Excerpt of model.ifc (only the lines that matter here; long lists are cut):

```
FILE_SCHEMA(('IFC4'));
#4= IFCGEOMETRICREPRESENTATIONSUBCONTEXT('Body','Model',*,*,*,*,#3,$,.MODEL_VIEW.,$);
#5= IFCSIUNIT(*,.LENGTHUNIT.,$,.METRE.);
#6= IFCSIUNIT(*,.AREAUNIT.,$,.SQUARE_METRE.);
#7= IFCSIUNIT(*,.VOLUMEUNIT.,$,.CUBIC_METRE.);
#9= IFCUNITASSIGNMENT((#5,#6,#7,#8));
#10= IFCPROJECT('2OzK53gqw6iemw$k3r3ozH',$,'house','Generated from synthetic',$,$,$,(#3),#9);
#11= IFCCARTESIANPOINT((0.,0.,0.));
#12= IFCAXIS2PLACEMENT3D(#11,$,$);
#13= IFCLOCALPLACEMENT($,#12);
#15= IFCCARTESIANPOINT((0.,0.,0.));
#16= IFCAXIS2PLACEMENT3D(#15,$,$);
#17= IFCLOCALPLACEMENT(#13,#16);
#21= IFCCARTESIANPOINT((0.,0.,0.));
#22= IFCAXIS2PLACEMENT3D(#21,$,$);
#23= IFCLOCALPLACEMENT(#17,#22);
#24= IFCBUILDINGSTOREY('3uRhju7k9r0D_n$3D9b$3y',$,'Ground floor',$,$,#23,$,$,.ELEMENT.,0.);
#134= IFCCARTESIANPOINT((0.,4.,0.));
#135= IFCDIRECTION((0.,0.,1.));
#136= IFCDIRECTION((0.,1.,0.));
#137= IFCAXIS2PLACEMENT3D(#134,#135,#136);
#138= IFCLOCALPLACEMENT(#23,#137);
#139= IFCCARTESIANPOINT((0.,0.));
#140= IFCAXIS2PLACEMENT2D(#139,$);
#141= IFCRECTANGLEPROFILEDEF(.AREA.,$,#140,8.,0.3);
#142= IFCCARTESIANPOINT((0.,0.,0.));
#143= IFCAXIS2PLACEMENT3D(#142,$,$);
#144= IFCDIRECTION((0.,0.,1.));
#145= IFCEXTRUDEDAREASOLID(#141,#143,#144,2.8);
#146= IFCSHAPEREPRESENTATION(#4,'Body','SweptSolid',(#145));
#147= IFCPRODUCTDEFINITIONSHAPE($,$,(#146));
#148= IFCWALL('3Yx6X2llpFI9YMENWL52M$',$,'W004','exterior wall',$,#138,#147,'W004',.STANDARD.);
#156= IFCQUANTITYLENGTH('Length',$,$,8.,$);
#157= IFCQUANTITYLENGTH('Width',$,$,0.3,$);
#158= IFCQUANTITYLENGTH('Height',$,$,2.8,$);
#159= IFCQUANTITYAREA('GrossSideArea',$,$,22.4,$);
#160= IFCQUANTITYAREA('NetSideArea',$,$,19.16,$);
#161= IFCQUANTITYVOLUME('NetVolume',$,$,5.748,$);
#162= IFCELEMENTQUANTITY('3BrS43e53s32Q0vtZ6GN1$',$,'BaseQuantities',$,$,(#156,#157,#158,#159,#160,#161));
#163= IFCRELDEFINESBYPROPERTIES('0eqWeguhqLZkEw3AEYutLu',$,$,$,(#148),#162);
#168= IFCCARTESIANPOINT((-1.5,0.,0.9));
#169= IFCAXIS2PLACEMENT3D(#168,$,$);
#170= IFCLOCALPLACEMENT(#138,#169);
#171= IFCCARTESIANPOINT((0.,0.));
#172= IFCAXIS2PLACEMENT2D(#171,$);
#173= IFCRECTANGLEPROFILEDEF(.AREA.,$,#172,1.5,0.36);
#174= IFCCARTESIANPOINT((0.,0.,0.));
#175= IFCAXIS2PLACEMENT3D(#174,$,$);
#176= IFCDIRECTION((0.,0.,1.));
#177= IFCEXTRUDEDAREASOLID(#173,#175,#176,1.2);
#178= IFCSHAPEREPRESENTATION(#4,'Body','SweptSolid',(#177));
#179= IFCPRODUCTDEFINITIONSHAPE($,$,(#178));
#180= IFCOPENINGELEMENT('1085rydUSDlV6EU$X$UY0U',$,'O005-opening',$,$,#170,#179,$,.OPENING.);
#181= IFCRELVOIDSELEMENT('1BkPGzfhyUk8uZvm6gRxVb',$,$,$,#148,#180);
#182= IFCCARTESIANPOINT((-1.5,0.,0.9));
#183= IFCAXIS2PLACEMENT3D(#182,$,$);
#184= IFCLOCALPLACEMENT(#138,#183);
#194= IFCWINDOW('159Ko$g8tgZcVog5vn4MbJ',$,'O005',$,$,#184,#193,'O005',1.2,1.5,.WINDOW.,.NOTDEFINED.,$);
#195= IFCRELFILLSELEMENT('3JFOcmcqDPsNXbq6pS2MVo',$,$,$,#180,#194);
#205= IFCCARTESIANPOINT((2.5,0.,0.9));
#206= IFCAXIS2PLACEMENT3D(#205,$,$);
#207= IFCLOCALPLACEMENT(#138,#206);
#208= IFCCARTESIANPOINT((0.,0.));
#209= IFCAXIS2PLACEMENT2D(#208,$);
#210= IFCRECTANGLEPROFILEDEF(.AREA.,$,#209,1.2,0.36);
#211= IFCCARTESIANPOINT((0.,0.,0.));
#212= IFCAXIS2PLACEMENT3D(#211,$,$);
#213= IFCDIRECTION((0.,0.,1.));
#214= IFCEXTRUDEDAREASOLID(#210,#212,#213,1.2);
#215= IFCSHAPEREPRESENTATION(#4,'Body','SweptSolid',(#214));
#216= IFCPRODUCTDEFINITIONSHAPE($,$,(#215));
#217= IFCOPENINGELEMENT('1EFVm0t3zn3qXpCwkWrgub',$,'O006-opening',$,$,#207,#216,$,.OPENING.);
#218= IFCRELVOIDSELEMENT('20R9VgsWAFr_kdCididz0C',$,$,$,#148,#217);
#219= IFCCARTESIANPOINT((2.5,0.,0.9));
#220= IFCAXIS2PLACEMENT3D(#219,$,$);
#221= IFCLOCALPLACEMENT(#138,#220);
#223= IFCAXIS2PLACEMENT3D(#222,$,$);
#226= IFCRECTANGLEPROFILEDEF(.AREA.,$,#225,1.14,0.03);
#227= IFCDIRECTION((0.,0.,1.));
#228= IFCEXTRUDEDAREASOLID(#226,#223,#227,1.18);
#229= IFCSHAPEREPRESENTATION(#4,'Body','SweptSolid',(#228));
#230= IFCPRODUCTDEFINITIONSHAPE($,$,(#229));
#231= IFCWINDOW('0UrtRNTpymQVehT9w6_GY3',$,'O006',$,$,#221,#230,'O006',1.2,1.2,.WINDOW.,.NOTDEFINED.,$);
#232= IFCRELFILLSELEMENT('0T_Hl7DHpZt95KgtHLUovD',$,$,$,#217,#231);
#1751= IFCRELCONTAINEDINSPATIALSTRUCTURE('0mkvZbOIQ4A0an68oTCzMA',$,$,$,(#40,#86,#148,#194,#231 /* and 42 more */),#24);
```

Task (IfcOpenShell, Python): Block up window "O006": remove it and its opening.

```python
import ifcopenshell
import ifcopenshell.api.feature
import ifcopenshell.api.pset
import ifcopenshell.api.root
import ifcopenshell.geom
import ifcopenshell.util.element
import ifcopenshell.util.shape
import ifcopenshell.util.unit

model = ifcopenshell.open("model.ifc")
area_scale = ifcopenshell.util.unit.calculate_unit_scale(model, "AREAUNIT")
volume_scale = ifcopenshell.util.unit.calculate_unit_scale(model, "VOLUMEUNIT")
settings = ifcopenshell.geom.settings()


def volume(element):
    """Net volume in cubic metres, openings subtracted."""
    shape = ifcopenshell.geom.create_shape(settings, element)
    return ifcopenshell.util.shape.get_volume(shape.geometry)


window = model.by_guid("0UrtRNTpymQVehT9w6_GY3")
opening = window.FillsVoids[0].RelatingOpeningElement
wall = opening.VoidsElements[0].RelatingBuildingElement
before = volume(wall)

ifcopenshell.api.root.remove_product(model, product=window)
ifcopenshell.api.feature.remove_feature(model, feature=opening)

after = volume(wall)
thickness = 0.3  # wall thickness in metres

# Update the wall's stored quantities.
qto = model.by_id(ifcopenshell.util.element.get_pset(wall, "BaseQuantities", should_inherit=False)["id"])
ifcopenshell.api.pset.edit_qto(model, qto=qto, properties={
    "NetSideArea": after / thickness / area_scale,
    "NetVolume": after / volume_scale,
})

print(f"wall volume {before:.3f} -> {after:.3f} m3")

model.write("model_edited.ifc")
```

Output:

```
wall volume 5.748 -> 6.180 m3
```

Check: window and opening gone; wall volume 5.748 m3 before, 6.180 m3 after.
